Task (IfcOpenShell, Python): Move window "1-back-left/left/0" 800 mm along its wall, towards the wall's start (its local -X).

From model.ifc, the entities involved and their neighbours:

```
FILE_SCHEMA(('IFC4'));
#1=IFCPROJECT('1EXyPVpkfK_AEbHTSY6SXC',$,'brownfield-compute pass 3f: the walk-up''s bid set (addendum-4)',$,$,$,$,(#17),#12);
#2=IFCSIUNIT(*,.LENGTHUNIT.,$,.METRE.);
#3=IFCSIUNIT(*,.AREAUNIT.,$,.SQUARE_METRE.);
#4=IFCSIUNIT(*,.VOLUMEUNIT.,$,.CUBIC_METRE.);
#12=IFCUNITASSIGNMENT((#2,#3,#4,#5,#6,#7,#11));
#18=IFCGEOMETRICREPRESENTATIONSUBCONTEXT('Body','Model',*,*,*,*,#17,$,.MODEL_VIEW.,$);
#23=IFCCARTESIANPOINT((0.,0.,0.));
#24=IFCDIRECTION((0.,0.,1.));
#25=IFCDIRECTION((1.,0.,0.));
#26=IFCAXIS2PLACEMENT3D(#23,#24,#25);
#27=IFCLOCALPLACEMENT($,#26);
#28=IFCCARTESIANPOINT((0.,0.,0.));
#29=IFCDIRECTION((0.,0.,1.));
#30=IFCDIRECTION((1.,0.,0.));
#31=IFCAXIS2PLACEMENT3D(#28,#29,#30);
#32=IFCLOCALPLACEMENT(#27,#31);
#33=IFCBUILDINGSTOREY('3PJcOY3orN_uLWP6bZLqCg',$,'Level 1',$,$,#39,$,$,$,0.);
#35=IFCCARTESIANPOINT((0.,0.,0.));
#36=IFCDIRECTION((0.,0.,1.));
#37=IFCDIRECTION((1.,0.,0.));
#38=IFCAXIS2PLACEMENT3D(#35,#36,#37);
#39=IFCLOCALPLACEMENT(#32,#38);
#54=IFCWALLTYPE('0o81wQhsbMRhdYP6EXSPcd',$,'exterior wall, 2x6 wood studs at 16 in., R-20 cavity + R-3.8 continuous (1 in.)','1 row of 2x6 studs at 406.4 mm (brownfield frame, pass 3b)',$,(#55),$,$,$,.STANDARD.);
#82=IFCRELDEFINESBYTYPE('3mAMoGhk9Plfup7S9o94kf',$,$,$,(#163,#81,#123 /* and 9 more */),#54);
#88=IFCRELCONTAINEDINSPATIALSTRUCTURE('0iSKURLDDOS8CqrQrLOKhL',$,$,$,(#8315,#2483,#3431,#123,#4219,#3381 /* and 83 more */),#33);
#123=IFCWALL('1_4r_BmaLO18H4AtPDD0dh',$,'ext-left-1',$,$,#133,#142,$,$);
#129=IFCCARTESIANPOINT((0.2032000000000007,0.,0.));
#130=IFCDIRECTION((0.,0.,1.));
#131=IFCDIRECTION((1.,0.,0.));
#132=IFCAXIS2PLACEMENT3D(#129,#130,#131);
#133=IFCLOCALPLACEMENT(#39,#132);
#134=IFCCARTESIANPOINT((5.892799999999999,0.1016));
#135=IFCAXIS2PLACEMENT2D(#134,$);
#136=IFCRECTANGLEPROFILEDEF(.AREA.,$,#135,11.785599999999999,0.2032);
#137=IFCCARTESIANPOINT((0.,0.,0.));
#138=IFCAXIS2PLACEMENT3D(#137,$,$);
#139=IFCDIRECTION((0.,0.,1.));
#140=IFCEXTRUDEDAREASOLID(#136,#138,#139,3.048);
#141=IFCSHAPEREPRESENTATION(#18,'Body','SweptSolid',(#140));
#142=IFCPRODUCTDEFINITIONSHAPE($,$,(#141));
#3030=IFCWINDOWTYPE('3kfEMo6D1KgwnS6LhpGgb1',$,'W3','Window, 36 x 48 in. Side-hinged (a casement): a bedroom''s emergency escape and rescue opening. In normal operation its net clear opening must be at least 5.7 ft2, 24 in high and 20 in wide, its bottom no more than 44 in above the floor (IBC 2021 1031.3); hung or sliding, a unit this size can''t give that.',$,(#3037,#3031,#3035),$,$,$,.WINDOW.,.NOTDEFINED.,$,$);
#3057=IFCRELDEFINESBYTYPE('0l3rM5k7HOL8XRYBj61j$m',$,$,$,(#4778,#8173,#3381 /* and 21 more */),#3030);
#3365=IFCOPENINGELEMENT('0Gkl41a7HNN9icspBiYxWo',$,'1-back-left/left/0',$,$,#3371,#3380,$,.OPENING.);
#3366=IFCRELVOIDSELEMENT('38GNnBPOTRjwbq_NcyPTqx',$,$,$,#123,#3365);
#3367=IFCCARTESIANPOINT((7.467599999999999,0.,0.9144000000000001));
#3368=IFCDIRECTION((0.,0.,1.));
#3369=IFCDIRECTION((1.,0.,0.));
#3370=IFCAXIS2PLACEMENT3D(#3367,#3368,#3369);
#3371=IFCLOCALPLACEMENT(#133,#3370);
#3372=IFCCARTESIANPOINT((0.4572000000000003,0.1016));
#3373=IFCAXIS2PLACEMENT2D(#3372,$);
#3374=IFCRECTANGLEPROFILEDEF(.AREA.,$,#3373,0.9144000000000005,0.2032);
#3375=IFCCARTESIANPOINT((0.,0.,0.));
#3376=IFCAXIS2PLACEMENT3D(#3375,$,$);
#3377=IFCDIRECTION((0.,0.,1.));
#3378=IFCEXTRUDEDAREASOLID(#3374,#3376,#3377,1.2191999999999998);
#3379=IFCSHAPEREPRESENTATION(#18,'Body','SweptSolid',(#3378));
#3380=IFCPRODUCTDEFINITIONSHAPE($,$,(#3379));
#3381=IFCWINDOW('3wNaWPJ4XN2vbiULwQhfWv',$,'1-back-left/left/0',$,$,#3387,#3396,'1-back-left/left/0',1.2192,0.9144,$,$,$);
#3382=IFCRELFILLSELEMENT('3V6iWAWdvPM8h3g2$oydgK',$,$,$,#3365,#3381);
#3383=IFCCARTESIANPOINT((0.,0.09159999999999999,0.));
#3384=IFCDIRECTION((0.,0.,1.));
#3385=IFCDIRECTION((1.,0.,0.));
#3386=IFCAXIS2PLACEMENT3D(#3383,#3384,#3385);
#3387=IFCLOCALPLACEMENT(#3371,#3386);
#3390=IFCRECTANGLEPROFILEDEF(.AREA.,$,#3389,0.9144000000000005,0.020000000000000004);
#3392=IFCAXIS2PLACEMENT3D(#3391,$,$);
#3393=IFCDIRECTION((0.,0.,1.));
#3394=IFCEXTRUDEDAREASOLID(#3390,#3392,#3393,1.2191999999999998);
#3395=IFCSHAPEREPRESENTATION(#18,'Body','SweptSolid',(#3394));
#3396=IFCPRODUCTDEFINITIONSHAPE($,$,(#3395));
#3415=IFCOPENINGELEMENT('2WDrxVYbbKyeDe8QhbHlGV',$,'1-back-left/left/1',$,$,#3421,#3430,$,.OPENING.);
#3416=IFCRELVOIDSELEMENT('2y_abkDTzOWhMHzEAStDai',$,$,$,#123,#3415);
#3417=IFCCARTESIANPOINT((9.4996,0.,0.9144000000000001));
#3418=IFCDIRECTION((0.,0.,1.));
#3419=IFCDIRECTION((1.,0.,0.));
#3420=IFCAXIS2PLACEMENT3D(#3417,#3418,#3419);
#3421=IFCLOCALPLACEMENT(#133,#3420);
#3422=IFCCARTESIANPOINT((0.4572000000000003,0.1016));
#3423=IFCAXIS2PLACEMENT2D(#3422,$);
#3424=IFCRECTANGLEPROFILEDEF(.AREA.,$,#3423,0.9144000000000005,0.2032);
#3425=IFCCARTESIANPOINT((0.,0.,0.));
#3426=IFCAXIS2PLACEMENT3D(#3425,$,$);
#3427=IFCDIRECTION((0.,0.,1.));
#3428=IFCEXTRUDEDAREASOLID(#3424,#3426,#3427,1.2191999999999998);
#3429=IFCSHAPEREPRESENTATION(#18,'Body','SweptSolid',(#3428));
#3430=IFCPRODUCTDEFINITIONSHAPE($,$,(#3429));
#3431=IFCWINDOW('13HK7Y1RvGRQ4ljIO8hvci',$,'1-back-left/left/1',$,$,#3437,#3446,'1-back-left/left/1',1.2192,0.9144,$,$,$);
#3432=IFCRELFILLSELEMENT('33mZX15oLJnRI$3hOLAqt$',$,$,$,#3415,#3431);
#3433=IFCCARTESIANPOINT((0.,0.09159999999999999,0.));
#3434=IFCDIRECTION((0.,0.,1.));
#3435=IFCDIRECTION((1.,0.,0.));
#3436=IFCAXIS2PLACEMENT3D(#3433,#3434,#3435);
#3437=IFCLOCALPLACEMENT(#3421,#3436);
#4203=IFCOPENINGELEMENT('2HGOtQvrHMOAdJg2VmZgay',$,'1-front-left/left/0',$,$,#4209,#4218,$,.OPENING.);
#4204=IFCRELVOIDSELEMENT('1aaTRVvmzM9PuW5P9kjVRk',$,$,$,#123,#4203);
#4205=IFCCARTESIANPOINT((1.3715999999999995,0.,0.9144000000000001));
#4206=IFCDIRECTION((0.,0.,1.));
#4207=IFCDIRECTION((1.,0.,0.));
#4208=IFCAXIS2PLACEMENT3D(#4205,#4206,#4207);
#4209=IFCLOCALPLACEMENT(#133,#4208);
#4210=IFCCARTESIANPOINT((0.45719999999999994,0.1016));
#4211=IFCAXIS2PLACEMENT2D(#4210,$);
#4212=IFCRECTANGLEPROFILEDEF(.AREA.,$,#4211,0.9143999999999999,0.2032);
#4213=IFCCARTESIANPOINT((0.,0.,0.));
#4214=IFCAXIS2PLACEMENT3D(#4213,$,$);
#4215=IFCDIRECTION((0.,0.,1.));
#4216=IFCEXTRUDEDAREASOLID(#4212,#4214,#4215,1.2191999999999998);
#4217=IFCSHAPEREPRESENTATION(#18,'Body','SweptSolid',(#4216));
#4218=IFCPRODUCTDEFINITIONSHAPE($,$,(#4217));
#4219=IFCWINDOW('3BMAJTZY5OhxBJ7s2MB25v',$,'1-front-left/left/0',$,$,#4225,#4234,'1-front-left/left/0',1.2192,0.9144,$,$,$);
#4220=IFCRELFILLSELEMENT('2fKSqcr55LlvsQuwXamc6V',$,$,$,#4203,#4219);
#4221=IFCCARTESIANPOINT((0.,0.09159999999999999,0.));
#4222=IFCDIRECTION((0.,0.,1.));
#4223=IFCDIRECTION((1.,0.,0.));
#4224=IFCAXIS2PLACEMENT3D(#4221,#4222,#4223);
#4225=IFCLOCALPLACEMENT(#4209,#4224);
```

```python
import ifcopenshell
import ifcopenshell.api.geometry
import ifcopenshell.util.placement

model = ifcopenshell.open("model.ifc")

window = model.by_guid("3wNaWPJ4XN2vbiULwQhfWv")
opening = window.FillsVoids[0].RelatingOpeningElement
wall = opening.VoidsElements[0].RelatingBuildingElement

wall_matrix = ifcopenshell.util.placement.get_local_placement(wall.ObjectPlacement)
shift = wall_matrix[:3, 0] * -0.8
before = ifcopenshell.util.placement.get_local_placement(window.ObjectPlacement)[:3, 3].copy()

# The window is placed relative to its opening, so it follows when the opening moves.
matrix = ifcopenshell.util.placement.get_local_placement(opening.ObjectPlacement)
matrix[:3, 3] += shift
ifcopenshell.api.geometry.edit_object_placement(
    model, product=opening, matrix=matrix, is_si=False, should_transform_children=True
)

after = ifcopenshell.util.placement.get_local_placement(window.ObjectPlacement)[:3, 3]
print("window moved by", (after - before).round(3) + 0.0)

model.write("model_updated.ifc")
```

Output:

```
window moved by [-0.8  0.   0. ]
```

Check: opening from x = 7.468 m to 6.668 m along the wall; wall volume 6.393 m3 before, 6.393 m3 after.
